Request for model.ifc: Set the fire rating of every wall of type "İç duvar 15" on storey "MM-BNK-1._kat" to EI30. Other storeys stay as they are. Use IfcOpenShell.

First a look at what the model holds.

```python
import ifcopenshell
import ifcopenshell.util.element

model = ifcopenshell.open("model.ifc")
print(model.schema)
storey = next(s for s in model.by_type("IfcBuildingStorey") if s.Name == "MM-BNK-1._kat")
walls = [e for e in ifcopenshell.util.element.get_decomposition(storey) if e.is_a("IfcWall")]
seen = {}
for e in walls:
    element_type = ifcopenshell.util.element.get_type(e)
    key = (element_type.Name if element_type != e and element_type else None, ifcopenshell.util.element.get_pset(e, "Pset_WallCommon", "FireRating"))
    seen[key] = seen.get(key, 0) + 1
for (name, value), count in sorted(seen.items(), key=str):
    print(count, "x", name, "|", value)
```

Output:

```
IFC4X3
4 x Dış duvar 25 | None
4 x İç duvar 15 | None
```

```python
import ifcopenshell
import ifcopenshell.api.pset
import ifcopenshell.util.element

model = ifcopenshell.open("model.ifc")

storey = next(s for s in model.by_type("IfcBuildingStorey") if s.Name == "MM-BNK-1._kat")
walls = [e for e in ifcopenshell.util.element.get_decomposition(storey) if e.is_a("IfcWall")]

count = 0
for e in walls:
    element_type = ifcopenshell.util.element.get_type(e)
    if element_type in (None, e) or element_type.Name != "İç duvar 15":
        continue
    # add_pset returns the element's existing set when there is one.
    pset = ifcopenshell.api.pset.add_pset(model, product=e, name="Pset_WallCommon")
    ifcopenshell.api.pset.edit_pset(model, pset=pset, properties={"FireRating": "EI30"})
    count += 1

print(count, "walls updated")

model.write("model-out.ifc")
```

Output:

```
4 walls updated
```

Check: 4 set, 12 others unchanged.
